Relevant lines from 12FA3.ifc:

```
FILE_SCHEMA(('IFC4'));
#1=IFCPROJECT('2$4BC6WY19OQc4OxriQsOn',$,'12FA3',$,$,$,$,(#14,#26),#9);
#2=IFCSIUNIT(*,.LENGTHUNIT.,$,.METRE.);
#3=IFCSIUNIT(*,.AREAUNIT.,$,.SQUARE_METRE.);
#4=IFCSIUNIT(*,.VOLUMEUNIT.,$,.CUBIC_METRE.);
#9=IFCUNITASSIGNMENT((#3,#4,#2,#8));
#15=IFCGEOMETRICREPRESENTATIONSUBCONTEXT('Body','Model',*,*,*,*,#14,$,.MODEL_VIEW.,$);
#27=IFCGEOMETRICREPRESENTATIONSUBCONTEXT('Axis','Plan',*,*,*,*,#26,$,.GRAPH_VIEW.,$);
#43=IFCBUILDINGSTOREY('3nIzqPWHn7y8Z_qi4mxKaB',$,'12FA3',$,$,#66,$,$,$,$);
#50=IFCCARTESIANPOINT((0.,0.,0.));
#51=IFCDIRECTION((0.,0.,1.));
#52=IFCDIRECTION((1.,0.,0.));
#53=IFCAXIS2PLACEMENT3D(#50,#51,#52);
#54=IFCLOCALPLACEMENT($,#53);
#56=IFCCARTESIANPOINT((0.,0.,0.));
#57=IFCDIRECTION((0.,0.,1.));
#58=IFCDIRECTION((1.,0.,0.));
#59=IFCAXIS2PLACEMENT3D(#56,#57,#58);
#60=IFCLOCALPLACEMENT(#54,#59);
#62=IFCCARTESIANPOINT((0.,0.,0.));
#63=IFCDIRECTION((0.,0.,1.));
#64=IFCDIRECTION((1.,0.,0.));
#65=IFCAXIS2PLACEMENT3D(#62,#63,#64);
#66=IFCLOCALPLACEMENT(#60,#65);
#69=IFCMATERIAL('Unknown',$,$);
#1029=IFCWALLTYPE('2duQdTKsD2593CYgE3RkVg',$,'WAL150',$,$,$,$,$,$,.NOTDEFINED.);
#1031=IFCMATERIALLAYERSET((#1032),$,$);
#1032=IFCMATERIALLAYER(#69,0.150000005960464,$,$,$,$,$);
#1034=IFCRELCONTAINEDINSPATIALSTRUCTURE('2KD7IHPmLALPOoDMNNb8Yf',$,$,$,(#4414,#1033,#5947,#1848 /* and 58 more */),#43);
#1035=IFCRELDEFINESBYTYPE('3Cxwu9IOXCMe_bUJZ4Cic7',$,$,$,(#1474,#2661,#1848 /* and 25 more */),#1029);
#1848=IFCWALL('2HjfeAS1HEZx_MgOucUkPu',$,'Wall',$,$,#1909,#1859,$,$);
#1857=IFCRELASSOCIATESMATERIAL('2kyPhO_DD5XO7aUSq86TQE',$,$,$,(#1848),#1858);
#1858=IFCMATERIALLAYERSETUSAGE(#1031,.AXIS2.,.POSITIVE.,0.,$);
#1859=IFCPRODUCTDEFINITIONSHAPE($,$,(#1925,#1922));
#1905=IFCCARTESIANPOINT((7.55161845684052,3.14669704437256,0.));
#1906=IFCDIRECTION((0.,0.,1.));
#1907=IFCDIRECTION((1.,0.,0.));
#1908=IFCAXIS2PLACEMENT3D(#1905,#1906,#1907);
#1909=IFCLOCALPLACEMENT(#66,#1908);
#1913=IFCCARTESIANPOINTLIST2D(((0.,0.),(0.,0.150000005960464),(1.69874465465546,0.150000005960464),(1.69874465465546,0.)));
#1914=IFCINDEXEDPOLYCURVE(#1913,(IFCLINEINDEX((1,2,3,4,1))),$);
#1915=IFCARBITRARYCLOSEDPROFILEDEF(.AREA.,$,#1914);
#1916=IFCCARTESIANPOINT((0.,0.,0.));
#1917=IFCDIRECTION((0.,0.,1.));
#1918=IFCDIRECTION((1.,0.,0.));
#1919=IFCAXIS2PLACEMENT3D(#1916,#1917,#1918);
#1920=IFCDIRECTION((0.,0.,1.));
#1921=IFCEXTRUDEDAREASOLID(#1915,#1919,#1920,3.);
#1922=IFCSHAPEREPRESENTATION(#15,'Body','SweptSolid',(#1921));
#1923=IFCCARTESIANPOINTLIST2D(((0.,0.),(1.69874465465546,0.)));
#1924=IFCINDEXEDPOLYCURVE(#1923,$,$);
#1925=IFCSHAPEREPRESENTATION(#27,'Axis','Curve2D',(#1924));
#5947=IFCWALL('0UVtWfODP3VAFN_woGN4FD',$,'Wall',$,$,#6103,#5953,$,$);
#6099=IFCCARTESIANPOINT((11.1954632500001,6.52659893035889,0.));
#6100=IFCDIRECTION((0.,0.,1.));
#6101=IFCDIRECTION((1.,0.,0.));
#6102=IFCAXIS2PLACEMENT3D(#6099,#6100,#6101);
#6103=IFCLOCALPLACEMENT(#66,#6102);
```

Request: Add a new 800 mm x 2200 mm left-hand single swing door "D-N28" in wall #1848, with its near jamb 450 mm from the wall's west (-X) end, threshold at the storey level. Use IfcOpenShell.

```python
import numpy as np
import ifcopenshell
import ifcopenshell.api.feature
import ifcopenshell.api.geometry
import ifcopenshell.api.root
import ifcopenshell.api.spatial
import ifcopenshell.geom
import ifcopenshell.util.element
import ifcopenshell.util.placement
import ifcopenshell.util.representation
import ifcopenshell.util.shape
import ifcopenshell.util.unit

model = ifcopenshell.open("12FA3.ifc")
unit_scale = ifcopenshell.util.unit.calculate_unit_scale(model)
settings = ifcopenshell.geom.settings()


def volume(element):
    """Net volume in cubic metres, openings subtracted."""
    shape = ifcopenshell.geom.create_shape(settings, element)
    return ifcopenshell.util.shape.get_volume(shape.geometry)


wall = model.by_id(1848)
storey = ifcopenshell.util.element.get_container(wall, ifc_class="IfcBuildingStorey")
context = ifcopenshell.util.representation.get_context(model, "Model", "Body", "MODEL_VIEW")
before = volume(wall)

width, height, from_end, sill = 0.8, 2.2, 0.45, 0.0  # metres

# The wall runs along its own X axis, and the end named is its -X end.
wall_shape = ifcopenshell.geom.create_shape(settings, wall)
x, y, z = ifcopenshell.util.shape.get_vertices(wall_shape.geometry).T
start = x.min() + from_end
face, thickness = float(y.min()), float(y.max() - y.min())
wall_matrix = ifcopenshell.util.placement.get_local_placement(wall.ObjectPlacement)
level = ifcopenshell.util.placement.get_local_placement(storey.ObjectPlacement)[2, 3]


def in_wall(x, y):
    """Placement at x, y metres in the wall's axes, at sill height."""
    matrix = wall_matrix.copy()
    matrix[:, 3] = wall_matrix @ np.array([x / unit_scale, y / unit_scale, 0.0, 1.0])
    matrix[2, 3] = level + sill / unit_scale
    return matrix


# Opening: a box that overshoots both wall faces by 50 mm.
opening = ifcopenshell.api.root.create_entity(model, ifc_class="IfcOpeningElement", predefined_type="OPENING")
box = ifcopenshell.api.geometry.add_wall_representation(
    model, context=context, length=width, height=height, thickness=thickness + 0.1
)
ifcopenshell.api.geometry.assign_representation(model, product=opening, representation=box)
ifcopenshell.api.geometry.edit_object_placement(model, product=opening, matrix=in_wall(start, face - 0.05), is_si=False)
ifcopenshell.api.feature.add_feature(model, feature=opening, element=wall)

door = ifcopenshell.api.root.create_entity(model, ifc_class="IfcDoor", name="D-N28", predefined_type="DOOR")
door.OverallWidth, door.OverallHeight = width / unit_scale, height / unit_scale
door.OperationType = "SINGLE_SWING_LEFT"
body = ifcopenshell.api.geometry.add_door_representation(
    model,
    context=context,
    overall_width=door.OverallWidth,
    overall_height=door.OverallHeight,
    operation_type="SINGLE_SWING_LEFT",
    lining_properties={"LiningDepth": thickness / unit_scale, "ThresholdDepth": thickness / unit_scale},
)
ifcopenshell.api.geometry.assign_representation(model, product=door, representation=body)
ifcopenshell.api.spatial.assign_container(model, products=[door], relating_structure=storey)
ifcopenshell.api.feature.add_filling(model, opening=opening, element=door)

# The lining spans the wall, so the door starts at the wall face.
ifcopenshell.api.geometry.edit_object_placement(model, product=door, matrix=in_wall(start, face), is_si=False)

after = volume(wall)

print(f"wall volume {before:.3f} -> {after:.3f} m3")

model.write("12FA3-out.ifc")
```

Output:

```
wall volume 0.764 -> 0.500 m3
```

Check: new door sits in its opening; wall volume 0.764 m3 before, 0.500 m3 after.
